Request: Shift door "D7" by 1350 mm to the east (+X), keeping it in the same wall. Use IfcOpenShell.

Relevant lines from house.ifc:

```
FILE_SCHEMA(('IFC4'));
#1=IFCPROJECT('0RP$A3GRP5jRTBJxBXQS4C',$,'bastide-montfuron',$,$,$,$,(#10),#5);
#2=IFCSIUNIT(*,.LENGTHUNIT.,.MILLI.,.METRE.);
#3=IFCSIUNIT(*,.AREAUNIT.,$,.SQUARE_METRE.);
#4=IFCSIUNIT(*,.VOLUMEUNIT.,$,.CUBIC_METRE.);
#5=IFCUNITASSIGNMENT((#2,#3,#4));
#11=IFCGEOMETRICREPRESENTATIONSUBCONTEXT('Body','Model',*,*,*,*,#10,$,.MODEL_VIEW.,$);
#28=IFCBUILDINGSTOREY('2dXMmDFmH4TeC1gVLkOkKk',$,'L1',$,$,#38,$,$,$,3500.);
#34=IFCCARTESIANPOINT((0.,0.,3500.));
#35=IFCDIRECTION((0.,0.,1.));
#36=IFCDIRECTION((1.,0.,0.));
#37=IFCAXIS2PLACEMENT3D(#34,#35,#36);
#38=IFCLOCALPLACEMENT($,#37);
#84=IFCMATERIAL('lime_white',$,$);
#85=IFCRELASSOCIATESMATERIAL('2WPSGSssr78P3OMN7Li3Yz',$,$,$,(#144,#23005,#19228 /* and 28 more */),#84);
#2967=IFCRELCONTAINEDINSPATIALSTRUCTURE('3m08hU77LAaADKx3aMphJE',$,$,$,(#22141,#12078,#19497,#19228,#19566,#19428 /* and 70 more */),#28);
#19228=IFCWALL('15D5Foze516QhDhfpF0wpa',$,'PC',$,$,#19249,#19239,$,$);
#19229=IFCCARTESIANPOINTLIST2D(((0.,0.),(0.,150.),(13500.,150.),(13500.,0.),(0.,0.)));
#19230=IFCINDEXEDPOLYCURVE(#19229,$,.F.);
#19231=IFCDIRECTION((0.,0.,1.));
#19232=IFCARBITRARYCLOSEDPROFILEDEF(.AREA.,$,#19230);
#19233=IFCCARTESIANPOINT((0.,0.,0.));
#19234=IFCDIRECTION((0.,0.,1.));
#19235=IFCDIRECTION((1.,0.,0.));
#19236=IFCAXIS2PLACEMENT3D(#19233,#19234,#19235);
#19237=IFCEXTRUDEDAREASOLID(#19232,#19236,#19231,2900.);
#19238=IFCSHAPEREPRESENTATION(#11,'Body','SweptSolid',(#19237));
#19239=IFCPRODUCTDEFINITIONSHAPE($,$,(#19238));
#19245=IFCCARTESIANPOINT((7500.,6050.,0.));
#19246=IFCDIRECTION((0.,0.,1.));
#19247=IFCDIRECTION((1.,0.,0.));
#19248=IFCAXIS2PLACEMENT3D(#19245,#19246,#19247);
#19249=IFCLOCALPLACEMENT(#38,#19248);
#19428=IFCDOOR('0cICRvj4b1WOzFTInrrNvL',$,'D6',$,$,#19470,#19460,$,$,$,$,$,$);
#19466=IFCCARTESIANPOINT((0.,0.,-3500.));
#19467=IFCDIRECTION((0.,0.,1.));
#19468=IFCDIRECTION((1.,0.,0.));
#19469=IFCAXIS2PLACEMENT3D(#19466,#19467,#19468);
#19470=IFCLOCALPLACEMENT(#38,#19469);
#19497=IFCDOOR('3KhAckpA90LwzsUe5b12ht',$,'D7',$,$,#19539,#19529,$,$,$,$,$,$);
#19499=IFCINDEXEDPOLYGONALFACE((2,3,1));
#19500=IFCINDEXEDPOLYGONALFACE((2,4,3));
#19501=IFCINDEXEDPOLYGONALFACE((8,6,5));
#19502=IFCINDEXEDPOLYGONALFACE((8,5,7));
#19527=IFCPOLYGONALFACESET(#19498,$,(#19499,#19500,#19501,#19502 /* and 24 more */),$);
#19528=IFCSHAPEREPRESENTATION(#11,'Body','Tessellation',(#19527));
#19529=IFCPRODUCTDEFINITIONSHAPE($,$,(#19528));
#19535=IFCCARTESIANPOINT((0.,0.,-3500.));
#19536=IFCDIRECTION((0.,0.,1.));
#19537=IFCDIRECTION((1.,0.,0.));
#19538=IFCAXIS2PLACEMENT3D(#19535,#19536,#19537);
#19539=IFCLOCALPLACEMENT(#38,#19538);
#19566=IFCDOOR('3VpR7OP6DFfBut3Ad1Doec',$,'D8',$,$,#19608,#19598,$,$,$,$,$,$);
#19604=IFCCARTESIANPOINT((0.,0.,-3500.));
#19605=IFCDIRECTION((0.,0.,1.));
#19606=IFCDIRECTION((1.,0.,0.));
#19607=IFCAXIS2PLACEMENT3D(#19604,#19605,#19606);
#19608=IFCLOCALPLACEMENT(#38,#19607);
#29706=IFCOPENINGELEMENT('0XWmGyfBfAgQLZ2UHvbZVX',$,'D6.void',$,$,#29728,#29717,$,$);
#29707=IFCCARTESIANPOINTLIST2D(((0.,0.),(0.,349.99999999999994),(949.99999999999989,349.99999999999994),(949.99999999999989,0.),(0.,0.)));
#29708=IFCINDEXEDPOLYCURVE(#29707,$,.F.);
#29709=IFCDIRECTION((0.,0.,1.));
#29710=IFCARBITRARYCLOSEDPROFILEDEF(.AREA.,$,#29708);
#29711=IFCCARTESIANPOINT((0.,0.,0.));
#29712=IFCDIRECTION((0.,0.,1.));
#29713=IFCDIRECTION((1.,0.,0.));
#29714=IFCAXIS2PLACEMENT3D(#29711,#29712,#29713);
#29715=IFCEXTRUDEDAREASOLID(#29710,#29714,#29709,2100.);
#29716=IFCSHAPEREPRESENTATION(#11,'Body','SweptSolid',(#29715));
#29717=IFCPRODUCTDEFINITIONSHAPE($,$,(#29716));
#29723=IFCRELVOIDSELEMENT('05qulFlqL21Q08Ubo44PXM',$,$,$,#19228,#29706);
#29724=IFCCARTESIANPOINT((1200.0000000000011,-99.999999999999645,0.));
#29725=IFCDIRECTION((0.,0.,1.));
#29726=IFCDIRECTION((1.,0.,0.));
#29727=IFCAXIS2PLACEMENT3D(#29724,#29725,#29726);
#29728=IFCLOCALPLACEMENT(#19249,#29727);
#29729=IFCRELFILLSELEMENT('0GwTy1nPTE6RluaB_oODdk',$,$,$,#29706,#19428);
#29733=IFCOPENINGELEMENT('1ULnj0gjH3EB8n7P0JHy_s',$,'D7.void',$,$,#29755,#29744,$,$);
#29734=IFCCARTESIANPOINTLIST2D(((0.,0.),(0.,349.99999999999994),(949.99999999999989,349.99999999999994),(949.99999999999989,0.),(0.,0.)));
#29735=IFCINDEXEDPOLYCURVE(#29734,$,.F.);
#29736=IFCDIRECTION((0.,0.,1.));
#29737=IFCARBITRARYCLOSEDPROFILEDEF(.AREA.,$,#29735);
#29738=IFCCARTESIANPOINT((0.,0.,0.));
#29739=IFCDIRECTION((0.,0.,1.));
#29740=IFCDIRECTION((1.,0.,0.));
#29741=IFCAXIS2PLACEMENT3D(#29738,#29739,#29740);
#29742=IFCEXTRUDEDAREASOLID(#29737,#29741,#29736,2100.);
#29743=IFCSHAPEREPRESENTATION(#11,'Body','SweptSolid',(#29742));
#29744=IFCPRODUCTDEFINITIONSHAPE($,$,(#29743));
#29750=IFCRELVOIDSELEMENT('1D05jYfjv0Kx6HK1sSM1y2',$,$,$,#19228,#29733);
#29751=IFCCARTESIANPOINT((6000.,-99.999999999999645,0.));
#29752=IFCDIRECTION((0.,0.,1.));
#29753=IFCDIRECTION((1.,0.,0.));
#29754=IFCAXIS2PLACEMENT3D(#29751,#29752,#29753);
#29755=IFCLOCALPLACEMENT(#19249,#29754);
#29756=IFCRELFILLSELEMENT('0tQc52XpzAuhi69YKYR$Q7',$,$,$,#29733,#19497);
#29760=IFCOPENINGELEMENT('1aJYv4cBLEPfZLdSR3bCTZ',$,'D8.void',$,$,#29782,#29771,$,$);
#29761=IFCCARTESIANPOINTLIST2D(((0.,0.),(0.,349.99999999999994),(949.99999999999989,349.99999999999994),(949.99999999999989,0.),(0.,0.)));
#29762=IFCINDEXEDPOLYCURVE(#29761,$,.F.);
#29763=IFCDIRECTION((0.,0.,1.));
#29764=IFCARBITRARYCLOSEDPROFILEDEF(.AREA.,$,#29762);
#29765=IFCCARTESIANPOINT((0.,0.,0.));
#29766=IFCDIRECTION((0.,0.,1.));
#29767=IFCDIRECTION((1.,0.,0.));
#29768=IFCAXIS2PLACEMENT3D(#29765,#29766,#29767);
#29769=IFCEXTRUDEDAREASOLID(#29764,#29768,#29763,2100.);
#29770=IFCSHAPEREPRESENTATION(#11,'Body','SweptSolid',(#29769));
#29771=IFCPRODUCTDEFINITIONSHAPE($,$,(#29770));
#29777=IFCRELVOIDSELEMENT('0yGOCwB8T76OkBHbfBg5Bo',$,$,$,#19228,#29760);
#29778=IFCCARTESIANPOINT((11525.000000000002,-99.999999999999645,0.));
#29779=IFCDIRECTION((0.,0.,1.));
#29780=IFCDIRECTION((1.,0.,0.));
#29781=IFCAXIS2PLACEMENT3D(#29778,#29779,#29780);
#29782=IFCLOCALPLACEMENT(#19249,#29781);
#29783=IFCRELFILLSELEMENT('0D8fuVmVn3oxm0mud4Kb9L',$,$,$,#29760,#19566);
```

```python
import ifcopenshell
import ifcopenshell.api.geometry
import ifcopenshell.util.placement
import ifcopenshell.util.unit

model = ifcopenshell.open("house.ifc")
unit_scale = ifcopenshell.util.unit.calculate_unit_scale(model)

door = model.by_id(19497)
opening = door.FillsVoids[0].RelatingOpeningElement
wall = opening.VoidsElements[0].RelatingBuildingElement

wall_matrix = ifcopenshell.util.placement.get_local_placement(wall.ObjectPlacement)
shift = wall_matrix[:3, 0] * 1.35 / unit_scale
before = ifcopenshell.util.placement.get_local_placement(door.ObjectPlacement)[:3, 3].copy()

# The door is not placed relative to its opening, so move both.
for product in (opening, door):
    matrix = ifcopenshell.util.placement.get_local_placement(product.ObjectPlacement)
    matrix[:3, 3] += shift
    ifcopenshell.api.geometry.edit_object_placement(model, product=product, matrix=matrix, is_si=False)

after = ifcopenshell.util.placement.get_local_placement(door.ObjectPlacement)[:3, 3]
print("door moved by", (after - before).round(3) + 0.0)

model.write("house_rev.ifc")
```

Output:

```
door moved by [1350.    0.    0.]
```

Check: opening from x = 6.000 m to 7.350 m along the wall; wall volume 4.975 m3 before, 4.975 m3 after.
